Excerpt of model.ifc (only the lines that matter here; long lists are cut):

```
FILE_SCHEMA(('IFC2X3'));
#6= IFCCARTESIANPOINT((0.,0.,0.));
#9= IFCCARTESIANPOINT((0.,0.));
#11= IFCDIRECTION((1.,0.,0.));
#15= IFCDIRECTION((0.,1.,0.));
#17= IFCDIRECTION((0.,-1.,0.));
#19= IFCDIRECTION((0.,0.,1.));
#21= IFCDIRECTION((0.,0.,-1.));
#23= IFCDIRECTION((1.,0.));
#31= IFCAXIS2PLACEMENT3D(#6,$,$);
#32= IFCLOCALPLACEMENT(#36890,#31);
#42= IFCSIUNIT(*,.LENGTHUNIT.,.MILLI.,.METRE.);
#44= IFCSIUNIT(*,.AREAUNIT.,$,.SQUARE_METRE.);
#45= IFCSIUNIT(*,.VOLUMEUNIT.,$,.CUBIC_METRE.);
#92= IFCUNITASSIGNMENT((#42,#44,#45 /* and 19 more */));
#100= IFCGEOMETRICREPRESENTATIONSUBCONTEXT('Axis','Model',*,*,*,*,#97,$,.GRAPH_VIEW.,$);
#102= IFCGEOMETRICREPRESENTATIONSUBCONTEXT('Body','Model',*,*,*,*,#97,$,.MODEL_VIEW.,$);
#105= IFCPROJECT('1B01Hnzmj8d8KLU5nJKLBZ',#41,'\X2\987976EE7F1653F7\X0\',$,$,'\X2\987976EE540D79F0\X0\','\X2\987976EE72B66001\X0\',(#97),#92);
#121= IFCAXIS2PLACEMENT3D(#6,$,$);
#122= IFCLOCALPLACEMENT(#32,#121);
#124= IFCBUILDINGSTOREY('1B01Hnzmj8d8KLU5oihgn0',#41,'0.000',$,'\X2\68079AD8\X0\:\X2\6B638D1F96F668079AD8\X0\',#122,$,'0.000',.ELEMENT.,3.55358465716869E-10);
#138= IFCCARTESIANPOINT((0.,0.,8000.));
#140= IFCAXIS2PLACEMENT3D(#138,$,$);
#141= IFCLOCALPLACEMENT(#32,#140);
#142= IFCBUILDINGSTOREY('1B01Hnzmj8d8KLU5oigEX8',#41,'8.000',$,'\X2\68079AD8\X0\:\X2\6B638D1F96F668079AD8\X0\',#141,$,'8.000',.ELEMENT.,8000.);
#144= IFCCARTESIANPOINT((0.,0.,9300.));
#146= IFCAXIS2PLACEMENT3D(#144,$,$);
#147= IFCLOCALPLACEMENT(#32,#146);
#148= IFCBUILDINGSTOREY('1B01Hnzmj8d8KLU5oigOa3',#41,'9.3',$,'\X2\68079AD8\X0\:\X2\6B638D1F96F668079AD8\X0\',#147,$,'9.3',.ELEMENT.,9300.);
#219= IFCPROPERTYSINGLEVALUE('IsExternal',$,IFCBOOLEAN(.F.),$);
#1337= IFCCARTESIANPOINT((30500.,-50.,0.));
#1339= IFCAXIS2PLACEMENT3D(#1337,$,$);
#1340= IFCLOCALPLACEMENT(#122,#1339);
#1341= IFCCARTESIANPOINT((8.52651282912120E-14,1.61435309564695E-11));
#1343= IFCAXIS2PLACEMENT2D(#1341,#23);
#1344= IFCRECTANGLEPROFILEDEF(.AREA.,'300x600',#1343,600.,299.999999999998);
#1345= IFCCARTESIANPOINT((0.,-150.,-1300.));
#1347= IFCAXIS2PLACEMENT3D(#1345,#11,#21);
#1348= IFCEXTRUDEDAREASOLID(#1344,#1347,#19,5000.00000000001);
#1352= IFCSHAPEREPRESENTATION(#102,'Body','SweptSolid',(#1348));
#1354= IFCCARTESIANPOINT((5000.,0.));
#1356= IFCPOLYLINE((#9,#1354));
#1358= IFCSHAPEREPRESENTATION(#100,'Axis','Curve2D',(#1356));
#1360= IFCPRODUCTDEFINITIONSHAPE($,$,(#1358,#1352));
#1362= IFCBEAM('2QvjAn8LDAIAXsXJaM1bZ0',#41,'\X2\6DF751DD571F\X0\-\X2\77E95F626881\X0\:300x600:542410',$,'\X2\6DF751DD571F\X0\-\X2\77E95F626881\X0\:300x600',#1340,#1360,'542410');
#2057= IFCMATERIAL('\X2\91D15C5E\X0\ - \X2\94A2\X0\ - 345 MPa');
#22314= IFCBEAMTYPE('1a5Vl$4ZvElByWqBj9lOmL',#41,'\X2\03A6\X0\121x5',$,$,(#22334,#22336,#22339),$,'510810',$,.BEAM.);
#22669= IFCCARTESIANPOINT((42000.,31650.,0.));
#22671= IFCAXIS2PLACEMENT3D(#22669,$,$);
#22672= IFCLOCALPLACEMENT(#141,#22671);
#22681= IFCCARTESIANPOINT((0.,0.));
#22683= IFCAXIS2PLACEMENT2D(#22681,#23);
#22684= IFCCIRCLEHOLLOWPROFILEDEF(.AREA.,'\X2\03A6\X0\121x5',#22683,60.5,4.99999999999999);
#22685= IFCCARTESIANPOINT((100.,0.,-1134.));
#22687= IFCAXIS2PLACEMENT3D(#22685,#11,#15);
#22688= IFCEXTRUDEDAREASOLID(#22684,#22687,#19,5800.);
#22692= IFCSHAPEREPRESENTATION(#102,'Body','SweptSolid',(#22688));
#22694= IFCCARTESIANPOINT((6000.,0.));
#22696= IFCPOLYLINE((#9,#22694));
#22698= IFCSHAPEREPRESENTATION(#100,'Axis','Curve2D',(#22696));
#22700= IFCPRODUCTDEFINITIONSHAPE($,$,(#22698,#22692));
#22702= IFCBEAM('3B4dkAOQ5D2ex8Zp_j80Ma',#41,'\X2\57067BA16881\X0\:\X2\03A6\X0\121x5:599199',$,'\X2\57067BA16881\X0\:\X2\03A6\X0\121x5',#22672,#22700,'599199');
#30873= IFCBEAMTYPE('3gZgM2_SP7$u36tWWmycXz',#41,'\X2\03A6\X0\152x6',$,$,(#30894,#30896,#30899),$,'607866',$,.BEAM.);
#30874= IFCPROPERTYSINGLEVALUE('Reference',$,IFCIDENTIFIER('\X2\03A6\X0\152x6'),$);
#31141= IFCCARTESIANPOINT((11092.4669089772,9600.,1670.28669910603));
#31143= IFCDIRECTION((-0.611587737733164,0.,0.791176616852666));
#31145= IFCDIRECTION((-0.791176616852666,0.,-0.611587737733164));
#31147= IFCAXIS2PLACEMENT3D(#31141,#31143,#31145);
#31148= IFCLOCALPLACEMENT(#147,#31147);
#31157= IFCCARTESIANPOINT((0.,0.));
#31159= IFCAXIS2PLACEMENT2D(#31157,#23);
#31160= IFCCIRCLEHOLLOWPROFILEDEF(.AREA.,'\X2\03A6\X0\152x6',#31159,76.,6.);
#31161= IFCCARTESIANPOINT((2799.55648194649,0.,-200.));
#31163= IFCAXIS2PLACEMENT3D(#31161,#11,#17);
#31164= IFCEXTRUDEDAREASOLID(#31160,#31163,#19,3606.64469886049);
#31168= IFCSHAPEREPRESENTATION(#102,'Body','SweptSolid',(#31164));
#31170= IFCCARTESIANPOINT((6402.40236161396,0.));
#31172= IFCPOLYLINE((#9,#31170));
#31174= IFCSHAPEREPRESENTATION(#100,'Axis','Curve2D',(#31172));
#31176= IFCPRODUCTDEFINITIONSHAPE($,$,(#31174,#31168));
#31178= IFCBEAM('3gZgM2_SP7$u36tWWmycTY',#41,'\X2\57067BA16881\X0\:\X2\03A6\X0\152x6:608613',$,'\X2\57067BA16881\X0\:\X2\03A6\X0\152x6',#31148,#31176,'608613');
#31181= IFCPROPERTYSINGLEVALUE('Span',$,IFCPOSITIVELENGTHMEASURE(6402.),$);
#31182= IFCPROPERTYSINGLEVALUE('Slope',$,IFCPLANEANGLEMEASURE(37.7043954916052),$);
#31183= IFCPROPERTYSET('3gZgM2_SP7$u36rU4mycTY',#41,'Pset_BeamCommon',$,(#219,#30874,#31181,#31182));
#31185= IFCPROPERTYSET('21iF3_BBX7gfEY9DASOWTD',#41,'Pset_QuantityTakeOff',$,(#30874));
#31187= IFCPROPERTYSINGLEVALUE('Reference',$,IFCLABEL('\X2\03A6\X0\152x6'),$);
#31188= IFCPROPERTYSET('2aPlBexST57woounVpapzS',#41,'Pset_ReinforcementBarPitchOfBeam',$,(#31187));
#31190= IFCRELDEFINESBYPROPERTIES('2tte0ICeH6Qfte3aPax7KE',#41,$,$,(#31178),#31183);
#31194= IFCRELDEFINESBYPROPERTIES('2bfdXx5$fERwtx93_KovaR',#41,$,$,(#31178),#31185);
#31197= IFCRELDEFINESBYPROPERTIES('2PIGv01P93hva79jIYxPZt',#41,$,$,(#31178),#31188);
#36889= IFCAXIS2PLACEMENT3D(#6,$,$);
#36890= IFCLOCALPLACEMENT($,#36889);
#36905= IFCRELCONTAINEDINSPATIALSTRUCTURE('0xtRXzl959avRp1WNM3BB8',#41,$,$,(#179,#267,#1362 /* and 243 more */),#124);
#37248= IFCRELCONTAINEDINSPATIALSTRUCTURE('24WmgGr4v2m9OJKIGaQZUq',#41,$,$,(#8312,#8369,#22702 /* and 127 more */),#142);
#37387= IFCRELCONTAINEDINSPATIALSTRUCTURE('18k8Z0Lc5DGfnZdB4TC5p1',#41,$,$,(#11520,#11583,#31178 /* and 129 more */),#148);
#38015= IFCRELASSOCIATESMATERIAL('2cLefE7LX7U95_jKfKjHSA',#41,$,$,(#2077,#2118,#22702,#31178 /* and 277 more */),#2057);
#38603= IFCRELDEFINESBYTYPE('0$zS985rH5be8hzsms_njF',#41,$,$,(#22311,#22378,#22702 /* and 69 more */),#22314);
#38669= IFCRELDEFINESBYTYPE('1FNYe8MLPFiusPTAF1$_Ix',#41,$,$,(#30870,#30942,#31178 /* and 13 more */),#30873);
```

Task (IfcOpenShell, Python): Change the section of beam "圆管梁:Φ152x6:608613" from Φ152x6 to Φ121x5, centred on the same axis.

```python
import ifcopenshell
import ifcopenshell.api.pset
import ifcopenshell.api.type
import ifcopenshell.util.element
import ifcopenshell.util.representation

model = ifcopenshell.open("model.ifc")

member = model.by_guid("3gZgM2_SP7$u36tWWmycTY")
source = next(p for p in model.by_type("IfcCircleHollowProfileDef") if p.ProfileName == "Φ121x5")

body = ifcopenshell.util.representation.get_representation(member, "Model", "Body")
solid = body.Items[0]
old_profile = solid.SweptArea

# Copy the section's sizes but keep this member's own profile position.
profile = ifcopenshell.util.element.copy(model, source)
profile.Position = old_profile.Position
solid.SweptArea = profile
if not model.get_total_inverses(old_profile):
    ifcopenshell.util.element.remove_deep2(model, old_profile)

new_type = model.by_guid("1a5Vl$4ZvElByWqBj9lOmL")
ifcopenshell.api.type.assign_type(
    model, related_objects=[member], relating_type=new_type, should_map_representations=False
)
member.Name = member.Name.replace("Φ152x6", "Φ121x5")
member.ObjectType = "圆管梁:Φ121x5"
pset = model.by_id(ifcopenshell.util.element.get_pset(member, "Pset_BeamCommon", should_inherit=False)["id"])
ifcopenshell.api.pset.edit_pset(model, pset=pset, properties={"Reference": "Φ121x5"})
pset = model.by_id(ifcopenshell.util.element.get_pset(member, "Pset_QuantityTakeOff", should_inherit=False)["id"])
ifcopenshell.api.pset.edit_pset(model, pset=pset, properties={"Reference": "Φ121x5"})
pset = model.by_id(ifcopenshell.util.element.get_pset(member, "Pset_ReinforcementBarPitchOfBeam", should_inherit=False)["id"])
ifcopenshell.api.pset.edit_pset(model, pset=pset, properties={"Reference": "Φ121x5"})

print(solid.SweptArea)

model.write("model_edited.ifc")
```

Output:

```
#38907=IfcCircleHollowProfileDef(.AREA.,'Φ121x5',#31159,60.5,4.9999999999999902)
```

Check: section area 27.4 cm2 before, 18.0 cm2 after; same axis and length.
